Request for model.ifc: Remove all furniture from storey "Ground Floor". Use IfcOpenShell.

First a look at what the model holds.

```python
import ifcopenshell
import ifcopenshell.util.element

model = ifcopenshell.open("model.ifc")
print(model.schema)
storey = next(s for s in model.by_type("IfcBuildingStorey") if s.Name == "Ground Floor")
furniture = [e for e in ifcopenshell.util.element.get_decomposition(storey) if e.is_a("IfcFurnishingElement")]
seen = {}
for e in furniture:
    element_type = ifcopenshell.util.element.get_type(e)
    name = element_type.Name if element_type not in (None, e) else None
    seen[name] = seen.get(name, 0) + 1
for name, count in sorted(seen.items(), key=str):
    print(count, "x", name)
```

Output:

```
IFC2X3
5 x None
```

```python
import ifcopenshell
import ifcopenshell.api.root
import ifcopenshell.util.element

model = ifcopenshell.open("model.ifc")

storey = next(s for s in model.by_type("IfcBuildingStorey") if s.Name == "Ground Floor")
furniture = [e for e in ifcopenshell.util.element.get_decomposition(storey) if e.is_a("IfcFurnishingElement")]

for e in furniture:
    ifcopenshell.api.root.remove_product(model, product=e)
print(len(furniture), "removed")

model.write("model-out.ifc")
```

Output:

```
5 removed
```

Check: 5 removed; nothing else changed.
